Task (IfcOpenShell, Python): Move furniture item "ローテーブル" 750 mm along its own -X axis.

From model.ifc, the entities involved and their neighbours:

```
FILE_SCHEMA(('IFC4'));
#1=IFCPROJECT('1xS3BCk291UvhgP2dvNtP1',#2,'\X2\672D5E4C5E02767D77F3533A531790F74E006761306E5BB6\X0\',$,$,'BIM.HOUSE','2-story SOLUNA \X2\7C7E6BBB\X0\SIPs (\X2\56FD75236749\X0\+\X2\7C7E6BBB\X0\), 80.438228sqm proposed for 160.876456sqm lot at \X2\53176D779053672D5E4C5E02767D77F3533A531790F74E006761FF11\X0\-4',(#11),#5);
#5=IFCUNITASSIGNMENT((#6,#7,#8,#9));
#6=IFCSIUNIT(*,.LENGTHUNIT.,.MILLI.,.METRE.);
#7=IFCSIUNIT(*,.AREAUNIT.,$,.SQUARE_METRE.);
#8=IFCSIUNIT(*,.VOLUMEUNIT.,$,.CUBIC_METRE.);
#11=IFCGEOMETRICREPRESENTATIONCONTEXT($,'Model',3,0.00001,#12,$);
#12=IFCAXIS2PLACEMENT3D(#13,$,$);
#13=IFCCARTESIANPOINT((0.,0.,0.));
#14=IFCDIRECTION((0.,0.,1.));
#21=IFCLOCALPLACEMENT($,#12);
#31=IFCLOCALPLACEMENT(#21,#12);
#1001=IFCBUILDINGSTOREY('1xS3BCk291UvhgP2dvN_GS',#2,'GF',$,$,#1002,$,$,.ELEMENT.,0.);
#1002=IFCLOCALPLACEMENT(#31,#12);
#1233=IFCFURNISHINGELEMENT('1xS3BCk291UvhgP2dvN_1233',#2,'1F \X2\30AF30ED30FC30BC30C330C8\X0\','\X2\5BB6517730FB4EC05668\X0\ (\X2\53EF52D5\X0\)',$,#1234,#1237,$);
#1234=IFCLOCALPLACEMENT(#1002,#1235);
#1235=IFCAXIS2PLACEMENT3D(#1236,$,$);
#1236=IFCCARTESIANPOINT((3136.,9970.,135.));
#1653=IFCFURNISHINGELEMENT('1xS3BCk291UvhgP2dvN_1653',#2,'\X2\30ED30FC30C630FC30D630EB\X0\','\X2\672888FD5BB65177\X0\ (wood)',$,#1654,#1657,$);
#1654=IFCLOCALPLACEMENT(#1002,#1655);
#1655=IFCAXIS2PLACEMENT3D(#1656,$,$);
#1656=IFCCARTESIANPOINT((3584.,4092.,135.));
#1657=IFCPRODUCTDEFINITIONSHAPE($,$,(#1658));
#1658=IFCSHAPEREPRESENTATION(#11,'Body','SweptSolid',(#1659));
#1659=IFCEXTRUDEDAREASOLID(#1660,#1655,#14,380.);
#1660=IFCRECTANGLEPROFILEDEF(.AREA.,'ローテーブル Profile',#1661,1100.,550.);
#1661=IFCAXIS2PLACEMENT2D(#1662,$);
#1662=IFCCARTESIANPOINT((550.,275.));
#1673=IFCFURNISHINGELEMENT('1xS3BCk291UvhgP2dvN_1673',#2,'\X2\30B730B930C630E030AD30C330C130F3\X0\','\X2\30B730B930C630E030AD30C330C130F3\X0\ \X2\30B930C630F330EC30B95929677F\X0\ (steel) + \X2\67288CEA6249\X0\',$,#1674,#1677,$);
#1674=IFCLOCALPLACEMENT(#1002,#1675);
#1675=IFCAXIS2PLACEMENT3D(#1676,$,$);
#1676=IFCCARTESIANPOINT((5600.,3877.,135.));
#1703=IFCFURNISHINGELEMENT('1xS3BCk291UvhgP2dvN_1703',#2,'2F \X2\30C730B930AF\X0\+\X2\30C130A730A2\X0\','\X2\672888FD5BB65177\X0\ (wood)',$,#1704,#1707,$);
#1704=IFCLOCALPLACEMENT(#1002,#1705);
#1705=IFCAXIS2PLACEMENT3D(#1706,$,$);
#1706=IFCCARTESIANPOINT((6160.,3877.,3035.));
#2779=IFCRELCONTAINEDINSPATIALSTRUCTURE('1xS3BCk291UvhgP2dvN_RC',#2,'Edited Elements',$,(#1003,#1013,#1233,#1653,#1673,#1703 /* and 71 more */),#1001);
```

```python
import ifcopenshell
import ifcopenshell.api.geometry
import ifcopenshell.util.placement

model = ifcopenshell.open("model.ifc")

item = model.by_guid("1xS3BCk291UvhgP2dvN_1653")
matrix = ifcopenshell.util.placement.get_local_placement(item.ObjectPlacement)
matrix[:3, 3] -= matrix[:3, 0] * 750.0
ifcopenshell.api.geometry.edit_object_placement(model, product=item, matrix=matrix, is_si=False)

print(ifcopenshell.util.placement.get_local_placement(item.ObjectPlacement).round(3) + 0.0)

model.write("model-out.ifc")
```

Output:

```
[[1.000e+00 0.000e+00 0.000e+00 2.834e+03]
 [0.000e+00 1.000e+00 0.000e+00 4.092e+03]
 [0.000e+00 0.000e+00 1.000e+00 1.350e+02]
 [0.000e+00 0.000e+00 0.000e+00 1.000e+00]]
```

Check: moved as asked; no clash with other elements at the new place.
